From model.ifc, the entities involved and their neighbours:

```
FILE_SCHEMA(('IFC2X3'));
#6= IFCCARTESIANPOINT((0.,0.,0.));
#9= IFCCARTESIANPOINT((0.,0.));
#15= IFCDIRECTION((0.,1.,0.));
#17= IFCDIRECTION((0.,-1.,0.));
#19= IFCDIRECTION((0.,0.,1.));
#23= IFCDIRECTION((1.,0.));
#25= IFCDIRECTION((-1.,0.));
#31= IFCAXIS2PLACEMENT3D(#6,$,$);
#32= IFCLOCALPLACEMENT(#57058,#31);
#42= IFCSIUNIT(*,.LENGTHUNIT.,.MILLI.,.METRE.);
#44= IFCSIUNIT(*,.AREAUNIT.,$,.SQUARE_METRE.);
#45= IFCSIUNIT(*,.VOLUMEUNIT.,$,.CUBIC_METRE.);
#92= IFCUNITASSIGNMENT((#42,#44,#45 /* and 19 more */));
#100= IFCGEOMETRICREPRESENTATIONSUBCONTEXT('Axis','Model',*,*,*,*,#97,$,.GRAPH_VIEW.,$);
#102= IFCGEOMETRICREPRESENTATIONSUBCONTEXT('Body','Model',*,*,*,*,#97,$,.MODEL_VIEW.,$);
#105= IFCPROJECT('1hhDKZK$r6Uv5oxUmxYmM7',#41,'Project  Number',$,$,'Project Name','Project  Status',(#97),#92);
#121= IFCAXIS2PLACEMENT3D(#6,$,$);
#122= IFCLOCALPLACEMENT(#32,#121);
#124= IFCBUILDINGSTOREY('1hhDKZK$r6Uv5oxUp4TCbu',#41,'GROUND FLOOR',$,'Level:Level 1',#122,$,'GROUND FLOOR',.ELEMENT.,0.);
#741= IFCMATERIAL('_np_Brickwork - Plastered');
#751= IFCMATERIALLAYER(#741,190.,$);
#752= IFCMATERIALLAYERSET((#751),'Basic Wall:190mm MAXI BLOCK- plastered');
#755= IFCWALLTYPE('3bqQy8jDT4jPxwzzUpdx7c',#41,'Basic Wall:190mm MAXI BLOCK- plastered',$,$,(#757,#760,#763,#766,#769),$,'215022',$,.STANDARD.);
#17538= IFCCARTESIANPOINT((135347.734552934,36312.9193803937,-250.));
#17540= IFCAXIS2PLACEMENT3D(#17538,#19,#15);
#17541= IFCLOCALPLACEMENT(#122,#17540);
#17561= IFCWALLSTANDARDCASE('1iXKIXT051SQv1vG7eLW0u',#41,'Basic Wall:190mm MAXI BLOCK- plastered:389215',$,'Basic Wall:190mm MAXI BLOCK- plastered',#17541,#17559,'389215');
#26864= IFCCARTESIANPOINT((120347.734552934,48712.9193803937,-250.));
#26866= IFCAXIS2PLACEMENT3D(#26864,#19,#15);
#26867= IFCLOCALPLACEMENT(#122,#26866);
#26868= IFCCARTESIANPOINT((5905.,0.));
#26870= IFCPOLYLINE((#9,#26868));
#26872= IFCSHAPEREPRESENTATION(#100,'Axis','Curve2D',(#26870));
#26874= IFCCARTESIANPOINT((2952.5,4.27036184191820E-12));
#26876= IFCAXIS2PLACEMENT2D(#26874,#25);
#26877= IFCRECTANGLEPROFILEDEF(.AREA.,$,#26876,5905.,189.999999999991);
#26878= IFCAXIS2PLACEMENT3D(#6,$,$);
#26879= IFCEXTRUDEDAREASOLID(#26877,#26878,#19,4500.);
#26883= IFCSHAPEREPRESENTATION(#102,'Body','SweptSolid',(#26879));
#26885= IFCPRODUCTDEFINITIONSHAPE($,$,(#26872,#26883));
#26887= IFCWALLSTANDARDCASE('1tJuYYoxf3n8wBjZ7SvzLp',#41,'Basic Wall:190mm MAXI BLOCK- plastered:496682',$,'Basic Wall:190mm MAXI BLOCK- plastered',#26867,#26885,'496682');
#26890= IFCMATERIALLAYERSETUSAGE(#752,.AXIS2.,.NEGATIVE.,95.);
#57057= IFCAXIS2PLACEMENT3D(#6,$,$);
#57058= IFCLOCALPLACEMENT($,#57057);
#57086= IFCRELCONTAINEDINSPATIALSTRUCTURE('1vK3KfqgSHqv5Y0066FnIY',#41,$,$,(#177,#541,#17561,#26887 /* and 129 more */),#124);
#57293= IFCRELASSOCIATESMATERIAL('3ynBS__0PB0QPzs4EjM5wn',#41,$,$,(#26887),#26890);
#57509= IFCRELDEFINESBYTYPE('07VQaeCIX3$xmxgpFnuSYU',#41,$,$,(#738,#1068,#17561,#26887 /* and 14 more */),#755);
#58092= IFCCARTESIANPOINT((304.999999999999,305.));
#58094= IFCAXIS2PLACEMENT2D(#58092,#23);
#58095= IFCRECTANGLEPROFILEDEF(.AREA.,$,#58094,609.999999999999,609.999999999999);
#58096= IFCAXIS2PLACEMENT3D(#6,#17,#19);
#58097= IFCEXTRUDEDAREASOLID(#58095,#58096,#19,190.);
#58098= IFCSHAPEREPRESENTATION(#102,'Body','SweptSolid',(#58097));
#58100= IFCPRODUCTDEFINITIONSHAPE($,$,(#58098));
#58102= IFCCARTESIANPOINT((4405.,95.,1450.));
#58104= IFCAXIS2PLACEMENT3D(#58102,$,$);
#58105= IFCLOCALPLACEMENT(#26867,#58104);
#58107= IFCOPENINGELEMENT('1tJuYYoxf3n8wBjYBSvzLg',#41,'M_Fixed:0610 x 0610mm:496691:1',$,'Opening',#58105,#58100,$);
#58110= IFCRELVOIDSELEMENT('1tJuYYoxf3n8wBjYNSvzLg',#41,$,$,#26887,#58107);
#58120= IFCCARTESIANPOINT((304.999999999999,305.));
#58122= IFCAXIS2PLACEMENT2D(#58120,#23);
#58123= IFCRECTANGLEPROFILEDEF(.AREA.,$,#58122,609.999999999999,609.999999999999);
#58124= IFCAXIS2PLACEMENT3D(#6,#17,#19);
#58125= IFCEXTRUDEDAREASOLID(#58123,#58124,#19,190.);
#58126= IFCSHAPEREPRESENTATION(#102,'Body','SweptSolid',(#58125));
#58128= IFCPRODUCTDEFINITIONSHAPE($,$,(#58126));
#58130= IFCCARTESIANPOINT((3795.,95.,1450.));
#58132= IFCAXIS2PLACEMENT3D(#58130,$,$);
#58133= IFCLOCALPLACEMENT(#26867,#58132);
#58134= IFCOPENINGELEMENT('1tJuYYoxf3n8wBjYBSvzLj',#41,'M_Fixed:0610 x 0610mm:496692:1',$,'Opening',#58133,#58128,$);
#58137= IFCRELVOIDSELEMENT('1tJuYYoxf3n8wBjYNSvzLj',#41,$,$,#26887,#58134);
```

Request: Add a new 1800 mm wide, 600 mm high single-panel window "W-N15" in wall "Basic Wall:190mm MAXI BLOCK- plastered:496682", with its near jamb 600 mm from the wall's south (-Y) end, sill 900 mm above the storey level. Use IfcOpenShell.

```python
import numpy as np
import ifcopenshell
import ifcopenshell.api.feature
import ifcopenshell.api.geometry
import ifcopenshell.api.root
import ifcopenshell.api.spatial
import ifcopenshell.api.type
import ifcopenshell.geom
import ifcopenshell.util.element
import ifcopenshell.util.placement
import ifcopenshell.util.representation
import ifcopenshell.util.shape
import ifcopenshell.util.unit

model = ifcopenshell.open("model.ifc")
unit_scale = ifcopenshell.util.unit.calculate_unit_scale(model)
settings = ifcopenshell.geom.settings()


def volume(element):
    """Net volume in cubic metres, openings subtracted."""
    shape = ifcopenshell.geom.create_shape(settings, element)
    return ifcopenshell.util.shape.get_volume(shape.geometry)


wall = model.by_guid("1tJuYYoxf3n8wBjZ7SvzLp")
storey = ifcopenshell.util.element.get_container(wall, ifc_class="IfcBuildingStorey")
context = ifcopenshell.util.representation.get_context(model, "Model", "Body", "MODEL_VIEW")
before = volume(wall)

width, height, from_end, sill = 1.8, 0.6, 0.6, 0.9  # metres

# The wall runs along its own X axis, and the end named is its -X end.
wall_shape = ifcopenshell.geom.create_shape(settings, wall)
x, y, z = ifcopenshell.util.shape.get_vertices(wall_shape.geometry).T
start = x.min() + from_end
face, thickness = float(y.min()), float(y.max() - y.min())
wall_matrix = ifcopenshell.util.placement.get_local_placement(wall.ObjectPlacement)
level = ifcopenshell.util.placement.get_local_placement(storey.ObjectPlacement)[2, 3]


def in_wall(x, y):
    """Placement at x, y metres in the wall's axes, at sill height."""
    matrix = wall_matrix.copy()
    matrix[:, 3] = wall_matrix @ np.array([x / unit_scale, y / unit_scale, 0.0, 1.0])
    matrix[2, 3] = level + sill / unit_scale
    return matrix


# Opening: a box that overshoots both wall faces by 50 mm.
opening = ifcopenshell.api.root.create_entity(model, ifc_class="IfcOpeningElement")
box = ifcopenshell.api.geometry.add_wall_representation(
    model, context=context, length=width, height=height, thickness=thickness + 0.1
)
ifcopenshell.api.geometry.assign_representation(model, product=opening, representation=box)
ifcopenshell.api.geometry.edit_object_placement(model, product=opening, matrix=in_wall(start, face - 0.05), is_si=False)
ifcopenshell.api.feature.add_feature(model, feature=opening, element=wall)

window = ifcopenshell.api.root.create_entity(model, ifc_class="IfcWindow", name="W-N15")
window.OverallWidth, window.OverallHeight = width / unit_scale, height / unit_scale
body = ifcopenshell.api.geometry.add_window_representation(
    model,
    context=context,
    overall_width=window.OverallWidth,
    overall_height=window.OverallHeight,
    partition_type="SINGLE_PANEL",
)
ifcopenshell.api.geometry.assign_representation(model, product=window, representation=body)
ifcopenshell.api.spatial.assign_container(model, products=[window], relating_structure=storey)
fills = ifcopenshell.api.feature.add_filling(model, opening=opening, element=window)
fills.OwnerHistory = window.OwnerHistory  # required in IFC2X3

# IFC2X3 keeps the operation on the window style.
style = ifcopenshell.api.root.create_entity(model, ifc_class="IfcWindowStyle", name="W-N15")
style.OperationType, style.ConstructionType = "SINGLE_PANEL", "NOTDEFINED"
style.ParameterTakesPrecedence = style.Sizeable = False
ifcopenshell.api.type.assign_type(model, related_objects=[window], relating_type=style)

# Centre the window in the wall's thickness.
ifcopenshell.api.geometry.edit_object_placement(model, product=window, matrix=in_wall(start, face), is_si=False)
window_shape = ifcopenshell.geom.create_shape(settings, window)
depth = ifcopenshell.util.shape.get_vertices(window_shape.geometry)[:, 1]
offset = face + thickness / 2 - (depth.min() + depth.max()) / 2
ifcopenshell.api.geometry.edit_object_placement(model, product=window, matrix=in_wall(start, offset), is_si=False)

after = volume(wall)

print(f"wall volume {before:.3f} -> {after:.3f} m3")

model.write("model_v2.ifc")
```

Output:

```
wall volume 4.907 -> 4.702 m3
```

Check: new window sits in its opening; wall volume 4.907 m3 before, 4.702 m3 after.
